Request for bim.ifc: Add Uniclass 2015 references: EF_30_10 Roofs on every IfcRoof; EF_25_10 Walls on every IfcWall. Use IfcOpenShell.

First a look at what the model holds.

```python
import ifcopenshell

model = ifcopenshell.open("bim.ifc")
print(model.schema)
print("classifications:", [c.Name for c in model.by_type("IfcClassification")])
for ifc_class in ("IfcDoor", "IfcRoof", "IfcStair", "IfcWall", "IfcWindow"):
    print(ifc_class, len(model.by_type(ifc_class)))
```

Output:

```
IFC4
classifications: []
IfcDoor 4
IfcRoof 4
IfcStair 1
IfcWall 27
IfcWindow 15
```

```python
import ifcopenshell
import ifcopenshell.api.classification

model = ifcopenshell.open("bim.ifc")

system = ifcopenshell.api.classification.add_classification(model, classification="Uniclass 2015")

codes = {
    "IfcRoof": ("EF_30_10", "Roofs"),
    "IfcWall": ("EF_25_10", "Walls"),
}
for ifc_class, (code, name) in codes.items():
    products = model.by_type(ifc_class)
    ifcopenshell.api.classification.add_reference(
        model, products=products, classification=system, identification=code, name=name
    )
    print(code, len(products))

model.write("bim_v2.ifc")
```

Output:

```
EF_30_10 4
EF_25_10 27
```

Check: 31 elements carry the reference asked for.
